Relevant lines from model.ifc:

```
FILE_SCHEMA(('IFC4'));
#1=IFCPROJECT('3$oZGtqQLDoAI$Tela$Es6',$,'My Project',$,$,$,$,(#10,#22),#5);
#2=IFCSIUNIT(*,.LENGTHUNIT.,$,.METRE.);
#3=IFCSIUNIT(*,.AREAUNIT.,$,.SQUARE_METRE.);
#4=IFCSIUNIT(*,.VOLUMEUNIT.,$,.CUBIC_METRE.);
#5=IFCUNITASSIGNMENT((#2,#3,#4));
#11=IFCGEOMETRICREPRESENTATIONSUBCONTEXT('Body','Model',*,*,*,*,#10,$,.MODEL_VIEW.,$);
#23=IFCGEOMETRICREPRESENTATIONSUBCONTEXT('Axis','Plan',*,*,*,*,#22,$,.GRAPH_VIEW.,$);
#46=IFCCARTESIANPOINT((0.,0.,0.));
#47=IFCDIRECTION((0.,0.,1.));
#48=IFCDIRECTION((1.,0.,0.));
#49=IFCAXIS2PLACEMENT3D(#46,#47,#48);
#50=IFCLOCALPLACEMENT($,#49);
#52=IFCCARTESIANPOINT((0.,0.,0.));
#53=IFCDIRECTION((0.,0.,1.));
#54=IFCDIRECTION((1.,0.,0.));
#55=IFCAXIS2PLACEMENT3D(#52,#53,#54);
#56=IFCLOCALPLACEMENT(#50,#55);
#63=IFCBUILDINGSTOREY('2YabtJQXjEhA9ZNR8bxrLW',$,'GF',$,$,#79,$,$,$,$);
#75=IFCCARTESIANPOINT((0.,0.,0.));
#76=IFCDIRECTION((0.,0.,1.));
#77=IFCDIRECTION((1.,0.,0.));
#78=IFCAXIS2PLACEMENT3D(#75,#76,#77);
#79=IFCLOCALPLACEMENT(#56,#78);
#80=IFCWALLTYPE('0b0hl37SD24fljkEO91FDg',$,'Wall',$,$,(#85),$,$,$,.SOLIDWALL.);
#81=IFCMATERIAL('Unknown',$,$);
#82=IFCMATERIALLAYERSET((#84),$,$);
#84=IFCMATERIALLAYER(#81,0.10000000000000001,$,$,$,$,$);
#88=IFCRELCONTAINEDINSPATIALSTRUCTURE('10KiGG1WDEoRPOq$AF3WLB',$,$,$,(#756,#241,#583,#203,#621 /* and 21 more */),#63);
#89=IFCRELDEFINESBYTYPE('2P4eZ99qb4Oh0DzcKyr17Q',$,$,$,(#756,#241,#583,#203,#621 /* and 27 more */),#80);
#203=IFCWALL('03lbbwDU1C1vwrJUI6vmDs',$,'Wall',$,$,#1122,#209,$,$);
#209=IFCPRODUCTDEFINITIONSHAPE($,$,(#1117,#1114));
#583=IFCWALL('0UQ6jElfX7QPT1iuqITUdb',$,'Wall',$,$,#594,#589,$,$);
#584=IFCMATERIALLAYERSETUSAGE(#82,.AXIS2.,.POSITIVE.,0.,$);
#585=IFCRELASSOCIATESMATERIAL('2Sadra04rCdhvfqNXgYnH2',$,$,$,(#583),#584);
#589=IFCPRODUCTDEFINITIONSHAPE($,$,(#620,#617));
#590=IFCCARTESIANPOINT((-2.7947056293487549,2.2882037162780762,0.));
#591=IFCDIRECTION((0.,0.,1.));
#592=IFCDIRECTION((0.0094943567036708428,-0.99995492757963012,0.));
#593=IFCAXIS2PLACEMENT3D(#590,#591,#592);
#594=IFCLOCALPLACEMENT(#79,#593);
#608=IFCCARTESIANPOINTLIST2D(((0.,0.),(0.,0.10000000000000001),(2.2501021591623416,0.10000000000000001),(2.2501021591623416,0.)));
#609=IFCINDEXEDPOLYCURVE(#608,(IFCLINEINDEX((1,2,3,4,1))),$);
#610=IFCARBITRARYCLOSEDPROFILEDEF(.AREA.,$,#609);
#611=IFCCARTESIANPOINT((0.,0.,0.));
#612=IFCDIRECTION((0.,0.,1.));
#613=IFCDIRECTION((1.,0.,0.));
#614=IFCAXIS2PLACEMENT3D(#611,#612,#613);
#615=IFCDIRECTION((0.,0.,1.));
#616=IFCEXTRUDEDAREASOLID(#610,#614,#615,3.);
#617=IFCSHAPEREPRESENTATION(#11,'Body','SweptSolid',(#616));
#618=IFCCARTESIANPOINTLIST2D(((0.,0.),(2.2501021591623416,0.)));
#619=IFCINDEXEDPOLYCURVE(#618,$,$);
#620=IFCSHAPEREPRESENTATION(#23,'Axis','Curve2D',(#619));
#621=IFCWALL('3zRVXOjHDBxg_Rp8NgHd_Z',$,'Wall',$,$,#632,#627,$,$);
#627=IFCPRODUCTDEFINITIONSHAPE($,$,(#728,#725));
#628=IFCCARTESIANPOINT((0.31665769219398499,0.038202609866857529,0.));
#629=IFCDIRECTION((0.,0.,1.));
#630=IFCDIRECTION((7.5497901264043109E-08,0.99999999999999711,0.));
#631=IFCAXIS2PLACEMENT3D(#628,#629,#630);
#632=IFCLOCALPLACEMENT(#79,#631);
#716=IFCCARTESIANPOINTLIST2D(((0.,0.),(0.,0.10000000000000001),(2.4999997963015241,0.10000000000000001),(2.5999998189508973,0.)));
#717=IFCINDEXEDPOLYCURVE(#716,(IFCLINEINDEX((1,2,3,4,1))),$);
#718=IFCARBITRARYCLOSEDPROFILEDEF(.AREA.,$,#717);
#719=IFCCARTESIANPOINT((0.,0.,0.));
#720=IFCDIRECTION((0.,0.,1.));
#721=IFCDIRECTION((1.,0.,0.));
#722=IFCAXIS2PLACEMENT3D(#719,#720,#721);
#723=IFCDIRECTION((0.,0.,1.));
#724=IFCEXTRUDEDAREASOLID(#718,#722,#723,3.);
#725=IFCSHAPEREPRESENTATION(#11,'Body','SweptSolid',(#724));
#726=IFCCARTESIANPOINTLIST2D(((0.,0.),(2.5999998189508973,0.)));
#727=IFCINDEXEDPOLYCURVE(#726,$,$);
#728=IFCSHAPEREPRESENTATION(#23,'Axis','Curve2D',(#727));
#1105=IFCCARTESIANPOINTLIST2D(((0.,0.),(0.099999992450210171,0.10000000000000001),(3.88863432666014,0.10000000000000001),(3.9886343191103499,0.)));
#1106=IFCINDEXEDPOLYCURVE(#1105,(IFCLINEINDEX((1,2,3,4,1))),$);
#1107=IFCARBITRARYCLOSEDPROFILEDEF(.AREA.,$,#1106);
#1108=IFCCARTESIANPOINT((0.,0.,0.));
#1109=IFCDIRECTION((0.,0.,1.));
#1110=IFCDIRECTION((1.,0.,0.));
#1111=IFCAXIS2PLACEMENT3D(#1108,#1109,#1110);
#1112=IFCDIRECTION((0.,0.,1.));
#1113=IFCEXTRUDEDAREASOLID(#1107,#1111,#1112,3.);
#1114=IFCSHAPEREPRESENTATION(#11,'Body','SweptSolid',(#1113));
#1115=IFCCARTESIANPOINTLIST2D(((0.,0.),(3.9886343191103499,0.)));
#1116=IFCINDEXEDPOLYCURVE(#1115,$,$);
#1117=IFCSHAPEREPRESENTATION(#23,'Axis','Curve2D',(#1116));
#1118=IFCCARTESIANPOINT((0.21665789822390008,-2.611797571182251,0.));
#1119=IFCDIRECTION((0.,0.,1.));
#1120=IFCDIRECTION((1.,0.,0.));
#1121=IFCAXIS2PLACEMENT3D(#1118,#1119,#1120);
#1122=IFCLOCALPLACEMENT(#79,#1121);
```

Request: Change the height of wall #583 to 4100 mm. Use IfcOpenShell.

```python
import ifcopenshell
import ifcopenshell.geom
import ifcopenshell.util.representation
import ifcopenshell.util.shape

model = ifcopenshell.open("model.ifc")
settings = ifcopenshell.geom.settings()


def volume(element):
    """Net volume in cubic metres, openings subtracted."""
    shape = ifcopenshell.geom.create_shape(settings, element)
    return ifcopenshell.util.shape.get_volume(shape.geometry)


wall = model.by_guid("0UQ6jElfX7QPT1iuqITUdb")
before = volume(wall)

body = ifcopenshell.util.representation.get_representation(wall, "Model", "Body")
solid = body.Items[0]
old_height = solid.Depth
solid.Depth = 4.1
after = volume(wall)

print(f"height {old_height:g} -> {solid.Depth:g}, volume {before:.3f} -> {after:.3f} m3")

model.write("model_updated.ifc")
```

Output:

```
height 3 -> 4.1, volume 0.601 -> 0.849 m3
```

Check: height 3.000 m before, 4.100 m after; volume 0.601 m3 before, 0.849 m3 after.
